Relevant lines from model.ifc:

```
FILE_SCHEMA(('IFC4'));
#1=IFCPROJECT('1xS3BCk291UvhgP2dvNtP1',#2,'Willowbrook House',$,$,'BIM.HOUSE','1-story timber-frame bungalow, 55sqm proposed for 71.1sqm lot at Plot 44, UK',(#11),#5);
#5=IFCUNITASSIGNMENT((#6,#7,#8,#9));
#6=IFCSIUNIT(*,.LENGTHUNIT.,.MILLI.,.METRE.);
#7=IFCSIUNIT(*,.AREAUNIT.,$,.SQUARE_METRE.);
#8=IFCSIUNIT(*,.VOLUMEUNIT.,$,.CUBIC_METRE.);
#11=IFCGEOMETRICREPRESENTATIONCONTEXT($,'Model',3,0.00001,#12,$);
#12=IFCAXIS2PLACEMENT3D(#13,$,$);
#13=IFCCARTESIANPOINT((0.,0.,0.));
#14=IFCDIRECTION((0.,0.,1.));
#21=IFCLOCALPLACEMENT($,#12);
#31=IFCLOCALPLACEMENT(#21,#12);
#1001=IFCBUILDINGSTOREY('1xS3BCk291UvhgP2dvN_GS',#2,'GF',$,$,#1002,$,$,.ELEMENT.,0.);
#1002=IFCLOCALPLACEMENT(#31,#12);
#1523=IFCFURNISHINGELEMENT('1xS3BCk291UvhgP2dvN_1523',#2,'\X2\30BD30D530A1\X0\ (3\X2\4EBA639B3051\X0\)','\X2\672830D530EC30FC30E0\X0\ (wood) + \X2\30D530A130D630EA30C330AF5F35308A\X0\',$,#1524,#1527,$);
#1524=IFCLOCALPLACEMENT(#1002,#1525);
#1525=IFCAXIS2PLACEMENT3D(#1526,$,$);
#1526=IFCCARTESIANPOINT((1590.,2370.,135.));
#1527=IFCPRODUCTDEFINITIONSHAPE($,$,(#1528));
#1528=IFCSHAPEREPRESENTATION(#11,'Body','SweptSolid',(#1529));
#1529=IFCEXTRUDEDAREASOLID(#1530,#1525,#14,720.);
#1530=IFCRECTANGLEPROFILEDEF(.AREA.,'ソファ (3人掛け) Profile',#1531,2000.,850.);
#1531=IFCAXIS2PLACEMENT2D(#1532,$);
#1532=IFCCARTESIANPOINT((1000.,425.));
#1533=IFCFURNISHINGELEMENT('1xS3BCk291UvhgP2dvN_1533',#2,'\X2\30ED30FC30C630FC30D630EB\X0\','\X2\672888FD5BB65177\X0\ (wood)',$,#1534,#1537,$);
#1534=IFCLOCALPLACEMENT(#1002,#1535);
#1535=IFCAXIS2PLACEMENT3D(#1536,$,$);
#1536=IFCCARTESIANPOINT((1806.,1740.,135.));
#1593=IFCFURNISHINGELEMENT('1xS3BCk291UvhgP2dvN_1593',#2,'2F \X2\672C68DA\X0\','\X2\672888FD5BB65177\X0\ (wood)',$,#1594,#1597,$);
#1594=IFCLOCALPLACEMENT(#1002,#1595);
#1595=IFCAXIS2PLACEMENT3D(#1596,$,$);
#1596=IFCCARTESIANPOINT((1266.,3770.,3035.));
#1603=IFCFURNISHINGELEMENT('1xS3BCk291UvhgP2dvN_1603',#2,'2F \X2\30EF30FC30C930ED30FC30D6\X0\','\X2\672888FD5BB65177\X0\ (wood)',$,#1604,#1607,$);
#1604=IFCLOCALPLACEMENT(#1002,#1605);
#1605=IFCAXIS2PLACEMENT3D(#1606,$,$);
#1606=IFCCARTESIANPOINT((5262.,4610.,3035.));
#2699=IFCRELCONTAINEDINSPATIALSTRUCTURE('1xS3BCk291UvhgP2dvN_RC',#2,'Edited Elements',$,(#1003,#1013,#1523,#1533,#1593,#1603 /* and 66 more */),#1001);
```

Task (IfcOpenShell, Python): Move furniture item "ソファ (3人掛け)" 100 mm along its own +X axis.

```python
import ifcopenshell
import ifcopenshell.api.geometry
import ifcopenshell.util.placement
import ifcopenshell.util.unit

model = ifcopenshell.open("model.ifc")
unit_scale = ifcopenshell.util.unit.calculate_unit_scale(model)

item = model.by_guid("1xS3BCk291UvhgP2dvN_1523")
matrix = ifcopenshell.util.placement.get_local_placement(item.ObjectPlacement)
matrix[:3, 3] += matrix[:3, 0] * 0.1 / unit_scale
ifcopenshell.api.geometry.edit_object_placement(model, product=item, matrix=matrix, is_si=False)

print(ifcopenshell.util.placement.get_local_placement(item.ObjectPlacement).round(3) + 0.0)

model.write("model_v2.ifc")
```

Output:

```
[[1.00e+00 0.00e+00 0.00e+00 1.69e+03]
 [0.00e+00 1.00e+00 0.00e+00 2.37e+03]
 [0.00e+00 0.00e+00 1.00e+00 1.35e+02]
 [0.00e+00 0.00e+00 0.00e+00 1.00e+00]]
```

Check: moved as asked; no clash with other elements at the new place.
